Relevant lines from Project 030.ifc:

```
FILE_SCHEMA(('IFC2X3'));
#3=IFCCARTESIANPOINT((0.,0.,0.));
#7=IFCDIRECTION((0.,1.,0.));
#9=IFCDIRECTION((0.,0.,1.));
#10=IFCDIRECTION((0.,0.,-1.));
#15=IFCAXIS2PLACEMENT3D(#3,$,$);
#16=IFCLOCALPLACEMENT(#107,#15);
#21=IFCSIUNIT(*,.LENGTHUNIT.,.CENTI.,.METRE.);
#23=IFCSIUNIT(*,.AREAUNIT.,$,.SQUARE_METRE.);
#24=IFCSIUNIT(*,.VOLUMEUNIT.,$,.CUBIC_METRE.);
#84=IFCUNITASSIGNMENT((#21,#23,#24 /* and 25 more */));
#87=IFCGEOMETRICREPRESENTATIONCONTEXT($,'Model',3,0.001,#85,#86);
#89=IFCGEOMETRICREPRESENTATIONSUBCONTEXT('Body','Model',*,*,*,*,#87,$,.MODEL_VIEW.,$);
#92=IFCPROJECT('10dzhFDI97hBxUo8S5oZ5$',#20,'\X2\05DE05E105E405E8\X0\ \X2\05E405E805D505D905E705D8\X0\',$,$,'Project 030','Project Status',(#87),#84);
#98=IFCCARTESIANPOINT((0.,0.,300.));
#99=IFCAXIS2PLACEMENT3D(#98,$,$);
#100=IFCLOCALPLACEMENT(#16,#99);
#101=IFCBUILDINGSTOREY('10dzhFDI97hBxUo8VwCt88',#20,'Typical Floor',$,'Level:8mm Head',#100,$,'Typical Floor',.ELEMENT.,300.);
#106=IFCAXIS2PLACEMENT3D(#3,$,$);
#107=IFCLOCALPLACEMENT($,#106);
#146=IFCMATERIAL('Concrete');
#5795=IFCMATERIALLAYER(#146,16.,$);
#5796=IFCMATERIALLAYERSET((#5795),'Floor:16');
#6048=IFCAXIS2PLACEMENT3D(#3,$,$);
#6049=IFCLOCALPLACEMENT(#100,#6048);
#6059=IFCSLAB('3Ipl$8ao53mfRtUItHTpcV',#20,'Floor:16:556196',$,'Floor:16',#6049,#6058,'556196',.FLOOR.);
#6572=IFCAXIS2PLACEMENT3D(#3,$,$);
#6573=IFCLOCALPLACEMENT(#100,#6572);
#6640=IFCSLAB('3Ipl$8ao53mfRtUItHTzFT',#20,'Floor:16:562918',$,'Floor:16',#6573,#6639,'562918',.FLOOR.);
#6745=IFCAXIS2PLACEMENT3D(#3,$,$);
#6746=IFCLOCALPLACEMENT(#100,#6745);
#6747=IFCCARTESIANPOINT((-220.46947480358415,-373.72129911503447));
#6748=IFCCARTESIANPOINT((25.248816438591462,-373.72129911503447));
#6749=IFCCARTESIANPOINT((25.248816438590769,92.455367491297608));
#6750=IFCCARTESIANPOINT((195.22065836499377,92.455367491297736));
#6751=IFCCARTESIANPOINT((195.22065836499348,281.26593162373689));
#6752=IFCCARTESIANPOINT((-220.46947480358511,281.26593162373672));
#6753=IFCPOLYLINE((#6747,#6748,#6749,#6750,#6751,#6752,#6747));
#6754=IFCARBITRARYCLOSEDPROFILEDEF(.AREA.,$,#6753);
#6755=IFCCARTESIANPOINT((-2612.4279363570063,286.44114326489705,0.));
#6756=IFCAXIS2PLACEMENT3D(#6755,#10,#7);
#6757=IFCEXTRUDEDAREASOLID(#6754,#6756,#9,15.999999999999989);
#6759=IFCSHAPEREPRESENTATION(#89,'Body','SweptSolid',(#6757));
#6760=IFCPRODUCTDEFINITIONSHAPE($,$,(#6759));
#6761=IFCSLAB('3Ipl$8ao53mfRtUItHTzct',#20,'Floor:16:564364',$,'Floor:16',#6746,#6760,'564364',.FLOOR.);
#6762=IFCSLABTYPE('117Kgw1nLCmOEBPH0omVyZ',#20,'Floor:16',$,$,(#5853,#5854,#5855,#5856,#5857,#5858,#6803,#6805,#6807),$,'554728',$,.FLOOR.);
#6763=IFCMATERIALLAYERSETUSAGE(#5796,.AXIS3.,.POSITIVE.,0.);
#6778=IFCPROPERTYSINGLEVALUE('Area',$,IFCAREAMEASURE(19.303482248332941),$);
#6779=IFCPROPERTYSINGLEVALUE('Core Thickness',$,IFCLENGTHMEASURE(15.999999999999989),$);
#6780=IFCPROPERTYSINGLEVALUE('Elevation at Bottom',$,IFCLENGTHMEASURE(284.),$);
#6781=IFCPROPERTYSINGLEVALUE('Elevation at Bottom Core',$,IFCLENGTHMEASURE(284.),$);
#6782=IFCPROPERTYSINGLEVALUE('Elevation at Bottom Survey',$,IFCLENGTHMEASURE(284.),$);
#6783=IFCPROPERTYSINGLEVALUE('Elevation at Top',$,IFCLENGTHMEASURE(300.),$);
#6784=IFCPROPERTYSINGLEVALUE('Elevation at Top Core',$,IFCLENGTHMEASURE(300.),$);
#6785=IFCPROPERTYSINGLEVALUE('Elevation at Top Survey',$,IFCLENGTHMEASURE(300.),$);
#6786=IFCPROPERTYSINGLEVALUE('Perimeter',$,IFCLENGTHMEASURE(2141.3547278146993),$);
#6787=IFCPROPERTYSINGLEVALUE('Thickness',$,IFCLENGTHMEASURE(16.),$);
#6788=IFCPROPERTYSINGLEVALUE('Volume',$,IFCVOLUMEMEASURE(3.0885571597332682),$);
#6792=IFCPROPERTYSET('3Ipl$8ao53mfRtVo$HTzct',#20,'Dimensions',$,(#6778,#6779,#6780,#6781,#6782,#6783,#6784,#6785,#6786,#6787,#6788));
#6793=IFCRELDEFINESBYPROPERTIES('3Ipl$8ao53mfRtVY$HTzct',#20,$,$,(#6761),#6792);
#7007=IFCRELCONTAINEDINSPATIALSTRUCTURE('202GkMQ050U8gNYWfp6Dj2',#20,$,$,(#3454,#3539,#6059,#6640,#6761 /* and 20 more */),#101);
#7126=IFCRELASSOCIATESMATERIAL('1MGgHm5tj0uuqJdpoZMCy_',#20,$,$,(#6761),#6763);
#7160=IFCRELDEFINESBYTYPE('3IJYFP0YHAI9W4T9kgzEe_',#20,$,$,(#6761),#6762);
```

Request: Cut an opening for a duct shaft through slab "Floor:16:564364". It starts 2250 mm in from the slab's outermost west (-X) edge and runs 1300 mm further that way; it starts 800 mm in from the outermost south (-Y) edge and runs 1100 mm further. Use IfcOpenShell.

```python
import numpy as np
import ifcopenshell
import ifcopenshell.api.feature
import ifcopenshell.api.geometry
import ifcopenshell.api.pset
import ifcopenshell.api.root
import ifcopenshell.geom
import ifcopenshell.util.element
import ifcopenshell.util.placement
import ifcopenshell.util.representation
import ifcopenshell.util.shape
import ifcopenshell.util.unit

model = ifcopenshell.open("Project 030.ifc")
unit_scale = ifcopenshell.util.unit.calculate_unit_scale(model)
area_scale = ifcopenshell.util.unit.calculate_unit_scale(model, "AREAUNIT")
volume_scale = ifcopenshell.util.unit.calculate_unit_scale(model, "VOLUMEUNIT")
settings = ifcopenshell.geom.settings()


def volume(element):
    """Net volume in cubic metres, openings subtracted."""
    shape = ifcopenshell.geom.create_shape(settings, element)
    return ifcopenshell.util.shape.get_volume(shape.geometry)


slab = model.by_id(6761)
before = volume(slab)

# Extent in the slab's own axes, in metres. The edges named are its -X and -Y sides.
slab_shape = ifcopenshell.geom.create_shape(settings, slab)
vertices = ifcopenshell.util.shape.get_vertices(slab_shape.geometry)
x_min, y_min, bottom = vertices.min(axis=0)
top = vertices[:, 2].max()

opening = ifcopenshell.api.root.create_entity(model, ifc_class="IfcOpeningElement", name="Duct shaft opening")
context = ifcopenshell.util.representation.get_context(model, "Model", "Body", "MODEL_VIEW")
width, depth = 1.3, 1.1
outline = [(0.0, 0.0), (width, 0.0), (width, depth), (0.0, depth), (0.0, 0.0)]
# Overshoot both faces by 50 mm so the cut is clean.
shape = ifcopenshell.api.geometry.add_slab_representation(
    model, context=context, depth=top - bottom + 0.1, polyline=outline
)
ifcopenshell.api.geometry.assign_representation(model, product=opening, representation=shape)

matrix = ifcopenshell.util.placement.get_local_placement(slab.ObjectPlacement)
matrix[:, 3] = matrix @ np.append(np.array([x_min + 2.25, y_min + 0.8, bottom - 0.05]) / unit_scale, 1.0)
ifcopenshell.api.geometry.edit_object_placement(model, product=opening, matrix=matrix, is_si=False)
ifcopenshell.api.feature.add_feature(model, feature=opening, element=slab)

after = volume(slab)

# Update the slab's stored quantities.
pset = model.by_id(ifcopenshell.util.element.get_pset(slab, "Dimensions", should_inherit=False)["id"])
ifcopenshell.api.pset.edit_pset(model, pset=pset, properties={
    "Area": model.create_entity("IfcAreaMeasure", after / (top - bottom) / area_scale),
    "Volume": model.create_entity("IfcVolumeMeasure", after / volume_scale),
})

print(f"slab volume {before:.3f} -> {after:.3f} m3")

model.write("Project 030_updated.ifc")
```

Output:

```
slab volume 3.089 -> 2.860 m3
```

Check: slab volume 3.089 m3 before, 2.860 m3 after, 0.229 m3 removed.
